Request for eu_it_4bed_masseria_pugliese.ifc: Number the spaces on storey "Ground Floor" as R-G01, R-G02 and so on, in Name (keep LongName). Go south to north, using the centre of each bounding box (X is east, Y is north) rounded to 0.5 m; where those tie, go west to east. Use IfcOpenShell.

First a look at what the model holds.

```python
import ifcopenshell
import ifcopenshell.util.element
import ifcopenshell.util.placement

model = ifcopenshell.open("eu_it_4bed_masseria_pugliese.ifc")
print(model.schema)
storey = next(s for s in model.by_type("IfcBuildingStorey") if s.Name == "Ground Floor")
spaces = [e for e in ifcopenshell.util.element.get_decomposition(storey) if e.is_a("IfcSpace")]
for e in sorted(spaces, key=lambda e: e.id()):
    origin = ifcopenshell.util.placement.get_local_placement(e.ObjectPlacement)[:3, 3]
    print(e.id(), e.Name, e.LongName, origin.round(2) + 0.0, sep=" | ")
```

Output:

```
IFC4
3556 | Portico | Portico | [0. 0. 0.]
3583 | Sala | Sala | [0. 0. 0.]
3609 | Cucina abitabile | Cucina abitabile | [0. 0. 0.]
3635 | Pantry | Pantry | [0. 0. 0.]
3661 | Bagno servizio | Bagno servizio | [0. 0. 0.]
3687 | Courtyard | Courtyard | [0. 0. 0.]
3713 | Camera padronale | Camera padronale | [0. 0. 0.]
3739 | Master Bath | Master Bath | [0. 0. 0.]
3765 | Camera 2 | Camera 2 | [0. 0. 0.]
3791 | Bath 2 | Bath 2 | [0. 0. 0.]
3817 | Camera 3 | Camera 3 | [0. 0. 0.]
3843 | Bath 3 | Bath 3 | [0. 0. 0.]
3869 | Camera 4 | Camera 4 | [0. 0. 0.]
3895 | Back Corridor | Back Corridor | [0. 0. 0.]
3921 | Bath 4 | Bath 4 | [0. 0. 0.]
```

```python
import ifcopenshell
import ifcopenshell.geom
import ifcopenshell.util.element
import ifcopenshell.util.shape

model = ifcopenshell.open("eu_it_4bed_masseria_pugliese.ifc")
settings = ifcopenshell.geom.settings()
settings.set("use-world-coords", True)


def centre(element):
    shape = ifcopenshell.geom.create_shape(settings, element)
    return ifcopenshell.util.shape.get_bbox_centroid(shape.geometry)


storey = next(s for s in model.by_type("IfcBuildingStorey") if s.Name == "Ground Floor")
spaces = [e for e in ifcopenshell.util.element.get_decomposition(storey) if e.is_a("IfcSpace")]

# Insertion points can sit at a corner or the storey origin, so sort by the geometry (in metres).
centres = {e: centre(e) for e in spaces}
spaces.sort(key=lambda e: (round(centres[e][1] / 0.5), centres[e][0]))

for i, e in enumerate(spaces, start=1):
    number = f"R-G{i:02d}"
    e.Name = number
    print(e.id(), number)

model.write("eu_it_4bed_masseria_pugliese_updated.ifc")
```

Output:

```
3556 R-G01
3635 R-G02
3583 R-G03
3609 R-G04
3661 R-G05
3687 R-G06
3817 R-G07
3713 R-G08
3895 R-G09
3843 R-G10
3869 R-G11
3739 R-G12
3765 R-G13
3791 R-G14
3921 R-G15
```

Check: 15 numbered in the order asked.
